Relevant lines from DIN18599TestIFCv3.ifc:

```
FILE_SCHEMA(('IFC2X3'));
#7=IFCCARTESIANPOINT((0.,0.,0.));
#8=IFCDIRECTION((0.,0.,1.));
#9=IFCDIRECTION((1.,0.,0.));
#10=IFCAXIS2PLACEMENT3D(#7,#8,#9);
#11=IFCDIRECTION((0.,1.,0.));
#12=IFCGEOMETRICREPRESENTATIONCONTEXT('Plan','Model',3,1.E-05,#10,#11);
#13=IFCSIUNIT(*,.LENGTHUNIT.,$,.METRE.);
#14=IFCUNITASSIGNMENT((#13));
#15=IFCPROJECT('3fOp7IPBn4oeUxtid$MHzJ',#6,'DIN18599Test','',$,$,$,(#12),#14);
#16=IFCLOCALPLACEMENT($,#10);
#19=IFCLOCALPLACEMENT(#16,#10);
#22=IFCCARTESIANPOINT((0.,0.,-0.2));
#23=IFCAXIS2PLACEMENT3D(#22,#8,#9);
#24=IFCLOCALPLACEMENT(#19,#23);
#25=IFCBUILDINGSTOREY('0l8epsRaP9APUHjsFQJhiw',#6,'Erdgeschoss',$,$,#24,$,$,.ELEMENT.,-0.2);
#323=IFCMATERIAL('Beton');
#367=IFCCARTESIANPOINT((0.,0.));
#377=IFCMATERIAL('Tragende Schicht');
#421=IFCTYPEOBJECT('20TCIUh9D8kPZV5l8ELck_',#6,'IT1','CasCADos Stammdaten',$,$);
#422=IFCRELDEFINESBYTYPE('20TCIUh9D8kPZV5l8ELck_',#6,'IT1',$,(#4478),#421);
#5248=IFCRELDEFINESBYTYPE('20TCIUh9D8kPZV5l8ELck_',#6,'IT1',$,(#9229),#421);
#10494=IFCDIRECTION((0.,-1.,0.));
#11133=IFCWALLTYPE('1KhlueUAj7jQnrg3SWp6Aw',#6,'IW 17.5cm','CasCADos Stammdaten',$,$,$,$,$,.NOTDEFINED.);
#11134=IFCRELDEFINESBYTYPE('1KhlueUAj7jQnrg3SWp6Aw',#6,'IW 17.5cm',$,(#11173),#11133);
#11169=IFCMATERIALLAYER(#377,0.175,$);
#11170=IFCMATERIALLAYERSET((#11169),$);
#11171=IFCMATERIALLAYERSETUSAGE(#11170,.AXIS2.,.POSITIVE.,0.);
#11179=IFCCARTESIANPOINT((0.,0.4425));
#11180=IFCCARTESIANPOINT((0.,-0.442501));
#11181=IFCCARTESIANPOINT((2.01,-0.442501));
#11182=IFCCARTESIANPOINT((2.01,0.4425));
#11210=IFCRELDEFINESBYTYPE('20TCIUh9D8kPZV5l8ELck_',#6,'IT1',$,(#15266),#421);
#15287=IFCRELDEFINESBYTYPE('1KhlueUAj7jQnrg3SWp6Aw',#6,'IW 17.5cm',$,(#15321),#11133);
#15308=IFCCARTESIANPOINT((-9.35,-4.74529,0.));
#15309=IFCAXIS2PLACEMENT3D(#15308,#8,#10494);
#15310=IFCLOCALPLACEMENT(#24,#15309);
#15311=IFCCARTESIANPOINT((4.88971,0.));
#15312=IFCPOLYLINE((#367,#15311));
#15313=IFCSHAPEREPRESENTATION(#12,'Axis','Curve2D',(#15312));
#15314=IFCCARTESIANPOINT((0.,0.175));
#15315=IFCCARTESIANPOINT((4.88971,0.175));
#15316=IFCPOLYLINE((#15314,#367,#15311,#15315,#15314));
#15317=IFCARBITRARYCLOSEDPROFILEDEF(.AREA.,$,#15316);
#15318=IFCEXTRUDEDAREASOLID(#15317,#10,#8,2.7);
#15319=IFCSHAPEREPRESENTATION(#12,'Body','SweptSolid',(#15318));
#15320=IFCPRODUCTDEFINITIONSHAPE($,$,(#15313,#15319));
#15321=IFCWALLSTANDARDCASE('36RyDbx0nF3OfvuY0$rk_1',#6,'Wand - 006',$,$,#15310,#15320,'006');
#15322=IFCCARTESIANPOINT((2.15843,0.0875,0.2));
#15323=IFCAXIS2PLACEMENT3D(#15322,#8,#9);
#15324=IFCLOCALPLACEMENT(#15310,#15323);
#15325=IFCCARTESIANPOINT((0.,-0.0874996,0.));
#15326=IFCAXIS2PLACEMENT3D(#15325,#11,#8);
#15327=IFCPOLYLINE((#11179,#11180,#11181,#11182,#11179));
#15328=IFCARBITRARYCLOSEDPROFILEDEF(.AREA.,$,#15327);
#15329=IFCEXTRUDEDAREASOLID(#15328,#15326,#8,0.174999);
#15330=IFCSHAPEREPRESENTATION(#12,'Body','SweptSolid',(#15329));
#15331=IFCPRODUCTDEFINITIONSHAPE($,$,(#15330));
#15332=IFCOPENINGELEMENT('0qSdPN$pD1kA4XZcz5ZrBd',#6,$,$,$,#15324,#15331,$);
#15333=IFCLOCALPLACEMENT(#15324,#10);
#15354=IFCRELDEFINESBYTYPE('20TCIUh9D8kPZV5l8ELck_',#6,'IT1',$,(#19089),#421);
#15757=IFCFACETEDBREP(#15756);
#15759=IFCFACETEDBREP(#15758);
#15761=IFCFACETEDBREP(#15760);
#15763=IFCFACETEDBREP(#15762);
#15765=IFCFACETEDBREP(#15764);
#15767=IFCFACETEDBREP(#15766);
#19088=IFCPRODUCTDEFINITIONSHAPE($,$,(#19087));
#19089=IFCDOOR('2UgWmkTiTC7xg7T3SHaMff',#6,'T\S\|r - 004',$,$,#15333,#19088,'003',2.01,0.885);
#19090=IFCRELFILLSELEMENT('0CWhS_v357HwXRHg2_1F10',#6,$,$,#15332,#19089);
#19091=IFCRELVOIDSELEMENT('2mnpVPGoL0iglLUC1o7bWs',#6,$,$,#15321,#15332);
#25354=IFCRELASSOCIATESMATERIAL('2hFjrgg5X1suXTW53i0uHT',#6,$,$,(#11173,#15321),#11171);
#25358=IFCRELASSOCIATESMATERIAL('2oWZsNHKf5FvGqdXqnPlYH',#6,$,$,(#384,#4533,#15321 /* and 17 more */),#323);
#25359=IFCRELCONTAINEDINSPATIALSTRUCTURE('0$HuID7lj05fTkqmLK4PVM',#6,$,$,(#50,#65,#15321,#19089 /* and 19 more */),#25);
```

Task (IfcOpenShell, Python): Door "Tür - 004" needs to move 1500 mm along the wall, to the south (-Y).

```python
import ifcopenshell
import ifcopenshell.api.geometry
import ifcopenshell.util.placement

model = ifcopenshell.open("DIN18599TestIFCv3.ifc")

door = model.by_guid("2UgWmkTiTC7xg7T3SHaMff")
opening = door.FillsVoids[0].RelatingOpeningElement
wall = opening.VoidsElements[0].RelatingBuildingElement

wall_matrix = ifcopenshell.util.placement.get_local_placement(wall.ObjectPlacement)
shift = wall_matrix[:3, 0] * 1.5
before = ifcopenshell.util.placement.get_local_placement(door.ObjectPlacement)[:3, 3].copy()

# The door is placed relative to its opening, so it follows when the opening moves.
matrix = ifcopenshell.util.placement.get_local_placement(opening.ObjectPlacement)
matrix[:3, 3] += shift
ifcopenshell.api.geometry.edit_object_placement(
    model, product=opening, matrix=matrix, is_si=False, should_transform_children=True
)

after = ifcopenshell.util.placement.get_local_placement(door.ObjectPlacement)[:3, 3]
print("door moved by", (after - before).round(3) + 0.0)

model.write("DIN18599TestIFCv3_rev.ifc")
```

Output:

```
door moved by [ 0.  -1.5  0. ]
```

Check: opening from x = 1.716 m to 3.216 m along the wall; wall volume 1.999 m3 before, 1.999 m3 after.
